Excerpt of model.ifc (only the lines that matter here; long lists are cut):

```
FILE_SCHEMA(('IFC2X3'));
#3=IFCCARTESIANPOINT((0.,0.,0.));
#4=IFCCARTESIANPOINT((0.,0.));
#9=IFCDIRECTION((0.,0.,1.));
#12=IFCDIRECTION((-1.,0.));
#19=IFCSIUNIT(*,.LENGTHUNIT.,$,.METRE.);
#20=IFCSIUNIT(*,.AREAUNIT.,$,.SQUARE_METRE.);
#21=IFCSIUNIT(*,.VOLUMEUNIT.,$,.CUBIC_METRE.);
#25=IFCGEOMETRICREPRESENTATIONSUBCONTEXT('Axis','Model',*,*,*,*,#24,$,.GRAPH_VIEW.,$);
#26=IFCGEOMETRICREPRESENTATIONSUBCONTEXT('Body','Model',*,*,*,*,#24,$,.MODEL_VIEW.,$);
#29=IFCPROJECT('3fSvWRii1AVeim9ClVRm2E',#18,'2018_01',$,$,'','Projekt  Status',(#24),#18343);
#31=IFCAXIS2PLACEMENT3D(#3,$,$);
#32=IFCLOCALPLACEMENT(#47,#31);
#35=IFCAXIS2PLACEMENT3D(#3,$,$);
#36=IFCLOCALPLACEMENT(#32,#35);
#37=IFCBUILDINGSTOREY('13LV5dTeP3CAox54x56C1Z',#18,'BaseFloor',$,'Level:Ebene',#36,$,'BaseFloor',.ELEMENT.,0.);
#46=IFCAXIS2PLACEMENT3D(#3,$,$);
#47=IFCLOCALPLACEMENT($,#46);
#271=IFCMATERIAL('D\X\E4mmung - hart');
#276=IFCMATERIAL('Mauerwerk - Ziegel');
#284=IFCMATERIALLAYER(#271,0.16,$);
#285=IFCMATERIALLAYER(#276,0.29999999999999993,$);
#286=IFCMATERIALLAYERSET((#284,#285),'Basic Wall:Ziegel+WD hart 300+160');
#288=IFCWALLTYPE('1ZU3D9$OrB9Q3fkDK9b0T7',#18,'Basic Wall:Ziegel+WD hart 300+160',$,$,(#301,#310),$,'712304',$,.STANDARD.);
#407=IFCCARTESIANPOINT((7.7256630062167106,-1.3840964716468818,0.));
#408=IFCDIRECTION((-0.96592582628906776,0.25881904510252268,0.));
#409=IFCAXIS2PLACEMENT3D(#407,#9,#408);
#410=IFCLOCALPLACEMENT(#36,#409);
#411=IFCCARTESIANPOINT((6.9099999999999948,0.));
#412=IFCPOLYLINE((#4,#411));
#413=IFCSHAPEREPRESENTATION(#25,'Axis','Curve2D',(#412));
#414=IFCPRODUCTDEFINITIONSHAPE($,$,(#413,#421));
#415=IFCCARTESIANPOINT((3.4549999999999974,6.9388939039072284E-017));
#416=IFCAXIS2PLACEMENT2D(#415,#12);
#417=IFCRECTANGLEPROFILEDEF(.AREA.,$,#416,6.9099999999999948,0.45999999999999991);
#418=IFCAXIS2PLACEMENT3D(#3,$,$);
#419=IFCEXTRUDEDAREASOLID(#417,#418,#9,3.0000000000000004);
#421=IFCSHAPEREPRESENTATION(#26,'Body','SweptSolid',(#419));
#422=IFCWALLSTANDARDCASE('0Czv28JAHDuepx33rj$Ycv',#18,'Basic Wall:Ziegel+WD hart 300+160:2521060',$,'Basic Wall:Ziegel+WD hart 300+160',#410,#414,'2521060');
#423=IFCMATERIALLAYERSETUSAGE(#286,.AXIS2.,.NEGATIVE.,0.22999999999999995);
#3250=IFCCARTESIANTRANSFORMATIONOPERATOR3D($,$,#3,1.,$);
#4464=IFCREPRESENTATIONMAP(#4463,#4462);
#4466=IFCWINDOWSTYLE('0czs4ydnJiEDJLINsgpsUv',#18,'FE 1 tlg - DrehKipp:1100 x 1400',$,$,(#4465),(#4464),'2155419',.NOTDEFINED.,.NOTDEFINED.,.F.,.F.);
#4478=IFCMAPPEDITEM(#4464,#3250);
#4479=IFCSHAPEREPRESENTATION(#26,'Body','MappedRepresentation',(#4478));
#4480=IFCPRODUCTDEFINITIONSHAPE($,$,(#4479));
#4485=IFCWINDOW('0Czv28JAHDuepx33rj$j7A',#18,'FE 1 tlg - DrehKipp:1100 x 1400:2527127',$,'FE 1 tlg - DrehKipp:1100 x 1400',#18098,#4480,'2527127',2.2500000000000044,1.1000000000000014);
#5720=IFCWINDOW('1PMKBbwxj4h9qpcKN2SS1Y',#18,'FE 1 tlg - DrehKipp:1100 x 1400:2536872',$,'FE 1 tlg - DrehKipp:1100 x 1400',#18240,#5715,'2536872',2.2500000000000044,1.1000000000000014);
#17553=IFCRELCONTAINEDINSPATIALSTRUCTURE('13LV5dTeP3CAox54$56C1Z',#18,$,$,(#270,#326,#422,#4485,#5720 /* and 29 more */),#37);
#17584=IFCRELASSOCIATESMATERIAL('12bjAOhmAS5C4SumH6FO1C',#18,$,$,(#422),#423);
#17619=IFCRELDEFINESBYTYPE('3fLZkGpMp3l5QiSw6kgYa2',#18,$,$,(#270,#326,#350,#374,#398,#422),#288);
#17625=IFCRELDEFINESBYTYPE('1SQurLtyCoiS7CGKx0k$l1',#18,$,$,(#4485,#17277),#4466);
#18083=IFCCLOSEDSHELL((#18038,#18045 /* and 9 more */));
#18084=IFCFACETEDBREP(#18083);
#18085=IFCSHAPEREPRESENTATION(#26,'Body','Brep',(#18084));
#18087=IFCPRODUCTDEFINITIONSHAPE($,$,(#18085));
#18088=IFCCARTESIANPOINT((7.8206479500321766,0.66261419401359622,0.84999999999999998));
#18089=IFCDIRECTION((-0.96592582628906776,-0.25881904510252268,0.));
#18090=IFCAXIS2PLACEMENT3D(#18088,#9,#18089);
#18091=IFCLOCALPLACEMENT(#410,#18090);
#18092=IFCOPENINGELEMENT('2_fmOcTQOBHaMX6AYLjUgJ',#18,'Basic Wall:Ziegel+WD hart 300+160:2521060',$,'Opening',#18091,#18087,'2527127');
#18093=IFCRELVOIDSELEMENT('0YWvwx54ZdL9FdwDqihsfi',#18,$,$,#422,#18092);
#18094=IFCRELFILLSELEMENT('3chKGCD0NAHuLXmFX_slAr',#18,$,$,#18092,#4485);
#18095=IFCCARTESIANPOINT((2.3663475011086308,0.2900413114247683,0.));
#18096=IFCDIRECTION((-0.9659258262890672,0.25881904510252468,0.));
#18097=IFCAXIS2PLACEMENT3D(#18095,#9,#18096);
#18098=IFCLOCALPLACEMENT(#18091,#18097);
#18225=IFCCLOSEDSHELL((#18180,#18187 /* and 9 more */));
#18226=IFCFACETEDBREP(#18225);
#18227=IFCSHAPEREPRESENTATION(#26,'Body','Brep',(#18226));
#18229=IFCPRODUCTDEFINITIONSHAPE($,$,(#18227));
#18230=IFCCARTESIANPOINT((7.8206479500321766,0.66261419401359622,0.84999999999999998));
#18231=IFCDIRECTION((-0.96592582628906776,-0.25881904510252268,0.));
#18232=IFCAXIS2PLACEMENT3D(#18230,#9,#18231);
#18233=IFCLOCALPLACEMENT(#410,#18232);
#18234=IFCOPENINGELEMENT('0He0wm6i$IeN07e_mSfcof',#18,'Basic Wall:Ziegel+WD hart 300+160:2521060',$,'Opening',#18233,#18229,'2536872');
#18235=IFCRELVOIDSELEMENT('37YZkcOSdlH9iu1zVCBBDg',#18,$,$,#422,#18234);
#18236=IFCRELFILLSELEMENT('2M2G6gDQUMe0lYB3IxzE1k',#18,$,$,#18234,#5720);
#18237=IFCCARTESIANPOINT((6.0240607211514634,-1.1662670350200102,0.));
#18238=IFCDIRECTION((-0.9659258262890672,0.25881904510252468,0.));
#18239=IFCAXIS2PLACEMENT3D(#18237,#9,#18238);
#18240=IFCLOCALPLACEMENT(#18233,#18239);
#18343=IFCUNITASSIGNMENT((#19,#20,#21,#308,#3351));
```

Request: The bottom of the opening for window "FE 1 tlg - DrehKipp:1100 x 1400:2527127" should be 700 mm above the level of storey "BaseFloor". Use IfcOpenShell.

```python
import numpy as np
import ifcopenshell
import ifcopenshell.api.geometry
import ifcopenshell.geom
import ifcopenshell.util.element
import ifcopenshell.util.placement
import ifcopenshell.util.shape
import ifcopenshell.util.unit

model = ifcopenshell.open("model.ifc")
unit_scale = ifcopenshell.util.unit.calculate_unit_scale(model)

window = model.by_id(4485)
opening = window.FillsVoids[0].RelatingOpeningElement
storey = ifcopenshell.util.element.get_container(window, ifc_class="IfcBuildingStorey")
level = ifcopenshell.util.placement.get_local_placement(storey.ObjectPlacement)[2, 3]

# The opening's origin need not be at the sill, so measure its lowest point.
shape = ifcopenshell.geom.create_shape(ifcopenshell.geom.settings(), opening)
bottom = ifcopenshell.util.shape.get_shape_bottom_elevation(shape, shape.geometry) / unit_scale
dz = level + 0.7 - bottom

shift = np.array([0.0, 0.0, dz])
# The window is placed relative to its opening, so it follows when the opening moves.
matrix = ifcopenshell.util.placement.get_local_placement(opening.ObjectPlacement)
matrix[:3, 3] += shift
ifcopenshell.api.geometry.edit_object_placement(
    model, product=opening, matrix=matrix, is_si=False, should_transform_children=True
)

print(f"moved by {dz * unit_scale:+.3f} m")

model.write("model-out.ifc")
```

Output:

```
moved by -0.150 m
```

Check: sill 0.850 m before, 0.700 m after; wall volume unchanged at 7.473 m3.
